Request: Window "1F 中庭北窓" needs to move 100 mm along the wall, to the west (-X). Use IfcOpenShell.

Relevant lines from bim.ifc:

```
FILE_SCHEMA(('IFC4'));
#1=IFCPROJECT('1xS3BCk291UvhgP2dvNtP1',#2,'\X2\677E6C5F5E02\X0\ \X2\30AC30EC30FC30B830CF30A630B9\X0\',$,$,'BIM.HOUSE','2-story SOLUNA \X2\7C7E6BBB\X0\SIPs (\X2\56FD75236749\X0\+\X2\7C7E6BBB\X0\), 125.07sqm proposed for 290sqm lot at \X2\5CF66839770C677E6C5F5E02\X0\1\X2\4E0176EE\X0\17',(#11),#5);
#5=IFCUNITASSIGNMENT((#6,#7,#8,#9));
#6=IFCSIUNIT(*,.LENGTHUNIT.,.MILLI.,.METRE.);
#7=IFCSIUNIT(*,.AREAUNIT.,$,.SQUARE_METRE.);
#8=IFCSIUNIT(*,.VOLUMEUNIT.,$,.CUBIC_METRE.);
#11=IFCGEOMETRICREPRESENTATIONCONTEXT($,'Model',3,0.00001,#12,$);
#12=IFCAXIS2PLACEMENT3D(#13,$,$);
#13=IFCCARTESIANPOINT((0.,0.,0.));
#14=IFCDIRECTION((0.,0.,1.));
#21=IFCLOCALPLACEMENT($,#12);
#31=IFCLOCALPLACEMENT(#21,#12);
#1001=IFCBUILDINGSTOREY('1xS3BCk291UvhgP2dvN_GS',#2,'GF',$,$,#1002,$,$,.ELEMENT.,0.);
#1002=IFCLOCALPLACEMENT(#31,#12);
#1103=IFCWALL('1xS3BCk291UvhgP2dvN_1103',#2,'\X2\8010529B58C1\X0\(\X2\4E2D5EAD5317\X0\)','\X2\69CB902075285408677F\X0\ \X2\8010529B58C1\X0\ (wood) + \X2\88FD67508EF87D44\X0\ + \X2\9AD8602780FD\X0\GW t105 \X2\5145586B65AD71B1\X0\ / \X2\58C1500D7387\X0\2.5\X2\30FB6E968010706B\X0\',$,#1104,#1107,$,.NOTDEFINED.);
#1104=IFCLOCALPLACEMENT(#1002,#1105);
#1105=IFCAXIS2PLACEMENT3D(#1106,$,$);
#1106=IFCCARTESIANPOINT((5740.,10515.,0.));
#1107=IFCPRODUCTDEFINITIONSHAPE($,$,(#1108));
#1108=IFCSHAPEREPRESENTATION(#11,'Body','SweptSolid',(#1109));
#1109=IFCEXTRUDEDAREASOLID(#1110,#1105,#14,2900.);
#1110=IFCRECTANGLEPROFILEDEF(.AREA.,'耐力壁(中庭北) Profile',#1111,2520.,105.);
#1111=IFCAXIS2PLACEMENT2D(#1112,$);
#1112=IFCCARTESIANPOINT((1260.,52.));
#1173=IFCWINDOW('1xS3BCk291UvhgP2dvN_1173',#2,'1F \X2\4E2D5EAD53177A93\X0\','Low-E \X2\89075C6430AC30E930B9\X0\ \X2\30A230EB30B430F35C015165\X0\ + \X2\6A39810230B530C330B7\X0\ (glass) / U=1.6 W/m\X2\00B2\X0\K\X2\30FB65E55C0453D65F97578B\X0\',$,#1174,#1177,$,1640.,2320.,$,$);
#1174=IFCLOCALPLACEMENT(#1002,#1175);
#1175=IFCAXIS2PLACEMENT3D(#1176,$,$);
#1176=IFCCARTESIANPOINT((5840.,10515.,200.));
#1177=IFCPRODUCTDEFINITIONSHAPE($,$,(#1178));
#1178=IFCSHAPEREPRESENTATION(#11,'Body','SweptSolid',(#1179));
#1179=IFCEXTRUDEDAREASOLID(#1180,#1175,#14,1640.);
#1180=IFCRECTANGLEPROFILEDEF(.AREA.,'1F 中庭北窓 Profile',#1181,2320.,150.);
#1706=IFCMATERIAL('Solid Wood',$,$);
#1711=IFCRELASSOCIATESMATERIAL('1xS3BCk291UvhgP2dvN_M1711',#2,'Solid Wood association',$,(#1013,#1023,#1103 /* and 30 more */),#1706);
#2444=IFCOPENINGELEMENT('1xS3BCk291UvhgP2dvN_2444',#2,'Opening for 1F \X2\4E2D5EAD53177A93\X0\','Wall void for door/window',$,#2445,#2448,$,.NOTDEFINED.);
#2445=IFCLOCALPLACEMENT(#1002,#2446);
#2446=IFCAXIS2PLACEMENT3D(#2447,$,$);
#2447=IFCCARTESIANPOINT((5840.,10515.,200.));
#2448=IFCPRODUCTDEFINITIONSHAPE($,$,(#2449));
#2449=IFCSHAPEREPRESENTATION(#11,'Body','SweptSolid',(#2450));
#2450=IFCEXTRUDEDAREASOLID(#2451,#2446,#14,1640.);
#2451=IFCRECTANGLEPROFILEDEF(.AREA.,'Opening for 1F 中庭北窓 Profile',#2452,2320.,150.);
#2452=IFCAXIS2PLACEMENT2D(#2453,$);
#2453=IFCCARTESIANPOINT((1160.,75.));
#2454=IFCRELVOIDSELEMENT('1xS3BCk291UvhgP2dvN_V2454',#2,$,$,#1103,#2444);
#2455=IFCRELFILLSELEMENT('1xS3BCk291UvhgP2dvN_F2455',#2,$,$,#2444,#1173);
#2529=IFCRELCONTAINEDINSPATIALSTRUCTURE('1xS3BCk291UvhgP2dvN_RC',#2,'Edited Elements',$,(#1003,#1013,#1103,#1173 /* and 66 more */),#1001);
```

```python
import ifcopenshell
import ifcopenshell.api.geometry
import ifcopenshell.util.placement
import ifcopenshell.util.unit

model = ifcopenshell.open("bim.ifc")
unit_scale = ifcopenshell.util.unit.calculate_unit_scale(model)

window = model.by_guid("1xS3BCk291UvhgP2dvN_1173")
opening = window.FillsVoids[0].RelatingOpeningElement
wall = opening.VoidsElements[0].RelatingBuildingElement

wall_matrix = ifcopenshell.util.placement.get_local_placement(wall.ObjectPlacement)
shift = wall_matrix[:3, 0] * -0.1 / unit_scale
before = ifcopenshell.util.placement.get_local_placement(window.ObjectPlacement)[:3, 3].copy()

# The window is not placed relative to its opening, so move both.
for product in (opening, window):
    matrix = ifcopenshell.util.placement.get_local_placement(product.ObjectPlacement)
    matrix[:3, 3] += shift
    ifcopenshell.api.geometry.edit_object_placement(model, product=product, matrix=matrix, is_si=False)

after = ifcopenshell.util.placement.get_local_placement(window.ObjectPlacement)[:3, 3]
print("window moved by", (after - before).round(3) + 0.0)

model.write("bim_updated.ifc")
```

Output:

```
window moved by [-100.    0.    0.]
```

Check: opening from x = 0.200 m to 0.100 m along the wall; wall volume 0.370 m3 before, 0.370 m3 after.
